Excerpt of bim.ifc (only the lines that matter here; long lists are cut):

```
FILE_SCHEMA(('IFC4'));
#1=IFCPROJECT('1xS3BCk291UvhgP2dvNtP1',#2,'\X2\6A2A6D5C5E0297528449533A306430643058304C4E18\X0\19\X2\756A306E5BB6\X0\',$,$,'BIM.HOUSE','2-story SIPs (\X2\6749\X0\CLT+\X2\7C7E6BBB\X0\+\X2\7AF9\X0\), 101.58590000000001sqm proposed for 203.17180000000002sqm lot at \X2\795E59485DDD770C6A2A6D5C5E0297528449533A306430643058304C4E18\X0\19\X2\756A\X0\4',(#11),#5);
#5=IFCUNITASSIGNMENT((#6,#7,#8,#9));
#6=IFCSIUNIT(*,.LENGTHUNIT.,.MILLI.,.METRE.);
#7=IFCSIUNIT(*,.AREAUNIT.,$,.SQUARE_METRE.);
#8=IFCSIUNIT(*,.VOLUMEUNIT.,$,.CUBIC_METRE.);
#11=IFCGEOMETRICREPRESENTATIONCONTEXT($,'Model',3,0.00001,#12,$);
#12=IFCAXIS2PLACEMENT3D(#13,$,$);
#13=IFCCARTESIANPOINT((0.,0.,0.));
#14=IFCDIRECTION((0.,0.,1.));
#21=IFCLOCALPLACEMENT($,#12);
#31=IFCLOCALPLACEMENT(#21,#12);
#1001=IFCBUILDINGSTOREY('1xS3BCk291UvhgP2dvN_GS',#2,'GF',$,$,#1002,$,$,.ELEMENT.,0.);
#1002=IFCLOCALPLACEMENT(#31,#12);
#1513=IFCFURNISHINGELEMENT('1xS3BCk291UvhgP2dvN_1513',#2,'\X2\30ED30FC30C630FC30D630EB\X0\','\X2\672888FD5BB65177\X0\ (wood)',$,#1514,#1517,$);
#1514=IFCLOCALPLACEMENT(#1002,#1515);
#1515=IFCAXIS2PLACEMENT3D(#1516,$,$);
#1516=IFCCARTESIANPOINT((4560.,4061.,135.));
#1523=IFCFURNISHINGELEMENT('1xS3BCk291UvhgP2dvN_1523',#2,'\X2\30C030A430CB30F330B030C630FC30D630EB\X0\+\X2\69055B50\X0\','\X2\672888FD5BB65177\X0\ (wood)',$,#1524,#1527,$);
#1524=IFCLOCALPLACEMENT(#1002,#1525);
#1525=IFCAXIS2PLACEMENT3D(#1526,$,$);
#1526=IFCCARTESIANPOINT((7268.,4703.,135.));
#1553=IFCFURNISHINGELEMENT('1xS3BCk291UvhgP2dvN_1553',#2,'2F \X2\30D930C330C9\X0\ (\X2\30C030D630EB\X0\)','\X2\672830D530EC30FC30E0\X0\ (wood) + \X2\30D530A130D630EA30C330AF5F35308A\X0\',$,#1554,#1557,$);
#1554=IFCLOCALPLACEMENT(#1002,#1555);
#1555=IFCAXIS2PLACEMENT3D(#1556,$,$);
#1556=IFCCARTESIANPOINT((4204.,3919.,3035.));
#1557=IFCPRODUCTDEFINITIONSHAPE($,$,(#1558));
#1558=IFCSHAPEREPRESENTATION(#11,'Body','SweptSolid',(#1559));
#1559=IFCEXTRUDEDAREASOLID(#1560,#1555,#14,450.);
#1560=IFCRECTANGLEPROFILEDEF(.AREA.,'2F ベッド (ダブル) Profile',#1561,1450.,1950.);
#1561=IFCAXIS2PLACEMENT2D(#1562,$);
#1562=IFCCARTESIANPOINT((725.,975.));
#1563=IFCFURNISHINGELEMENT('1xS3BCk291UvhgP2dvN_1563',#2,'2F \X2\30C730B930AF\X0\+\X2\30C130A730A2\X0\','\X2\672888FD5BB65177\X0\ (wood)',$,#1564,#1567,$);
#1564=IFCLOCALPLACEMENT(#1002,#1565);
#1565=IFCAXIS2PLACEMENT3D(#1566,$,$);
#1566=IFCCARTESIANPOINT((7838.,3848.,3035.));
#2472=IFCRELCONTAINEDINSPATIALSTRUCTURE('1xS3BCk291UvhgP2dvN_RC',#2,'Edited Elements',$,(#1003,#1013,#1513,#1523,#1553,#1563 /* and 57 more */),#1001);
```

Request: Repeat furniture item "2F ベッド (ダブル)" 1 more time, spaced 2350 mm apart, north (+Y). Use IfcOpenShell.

```python
import numpy as np
import ifcopenshell
import ifcopenshell.api.geometry
import ifcopenshell.api.root
import ifcopenshell.util.element
import ifcopenshell.util.placement
import ifcopenshell.util.unit

model = ifcopenshell.open("bim.ifc")
unit_scale = ifcopenshell.util.unit.calculate_unit_scale(model)


def reuse_history(source, copy):
    """copy_class also copies each property set's owner history, people and application; keep the originals."""
    for rel in copy.IsDefinedBy:
        if rel.is_a("IfcRelDefinesByProperties") and (history := rel.RelatingPropertyDefinition.OwnerHistory):
            rel.RelatingPropertyDefinition.OwnerHistory = source.OwnerHistory
            ifcopenshell.util.element.remove_deep2(model, history)


source = model.by_id(1553)
base = ifcopenshell.util.placement.get_local_placement(source.ObjectPlacement)
step = np.array([0.0, 1.0, 0.0]) * 2.35 / unit_scale

for i in range(1, 2):
    copy = ifcopenshell.api.root.copy_class(model, product=source)
    copy.Representation = ifcopenshell.util.element.copy_deep(
        model, source.Representation, exclude=["IfcGeometricRepresentationContext", "IfcRepresentationMap"]
    )
    reuse_history(source, copy)
    matrix = base.copy()
    matrix[:3, 3] += i * step
    print("added at", matrix[:3, 3].round(3) + 0.0)
    ifcopenshell.api.geometry.edit_object_placement(model, product=copy, matrix=matrix, is_si=False)

model.write("bim_edited.ifc")
```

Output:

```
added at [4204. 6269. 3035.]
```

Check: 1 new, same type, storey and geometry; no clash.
